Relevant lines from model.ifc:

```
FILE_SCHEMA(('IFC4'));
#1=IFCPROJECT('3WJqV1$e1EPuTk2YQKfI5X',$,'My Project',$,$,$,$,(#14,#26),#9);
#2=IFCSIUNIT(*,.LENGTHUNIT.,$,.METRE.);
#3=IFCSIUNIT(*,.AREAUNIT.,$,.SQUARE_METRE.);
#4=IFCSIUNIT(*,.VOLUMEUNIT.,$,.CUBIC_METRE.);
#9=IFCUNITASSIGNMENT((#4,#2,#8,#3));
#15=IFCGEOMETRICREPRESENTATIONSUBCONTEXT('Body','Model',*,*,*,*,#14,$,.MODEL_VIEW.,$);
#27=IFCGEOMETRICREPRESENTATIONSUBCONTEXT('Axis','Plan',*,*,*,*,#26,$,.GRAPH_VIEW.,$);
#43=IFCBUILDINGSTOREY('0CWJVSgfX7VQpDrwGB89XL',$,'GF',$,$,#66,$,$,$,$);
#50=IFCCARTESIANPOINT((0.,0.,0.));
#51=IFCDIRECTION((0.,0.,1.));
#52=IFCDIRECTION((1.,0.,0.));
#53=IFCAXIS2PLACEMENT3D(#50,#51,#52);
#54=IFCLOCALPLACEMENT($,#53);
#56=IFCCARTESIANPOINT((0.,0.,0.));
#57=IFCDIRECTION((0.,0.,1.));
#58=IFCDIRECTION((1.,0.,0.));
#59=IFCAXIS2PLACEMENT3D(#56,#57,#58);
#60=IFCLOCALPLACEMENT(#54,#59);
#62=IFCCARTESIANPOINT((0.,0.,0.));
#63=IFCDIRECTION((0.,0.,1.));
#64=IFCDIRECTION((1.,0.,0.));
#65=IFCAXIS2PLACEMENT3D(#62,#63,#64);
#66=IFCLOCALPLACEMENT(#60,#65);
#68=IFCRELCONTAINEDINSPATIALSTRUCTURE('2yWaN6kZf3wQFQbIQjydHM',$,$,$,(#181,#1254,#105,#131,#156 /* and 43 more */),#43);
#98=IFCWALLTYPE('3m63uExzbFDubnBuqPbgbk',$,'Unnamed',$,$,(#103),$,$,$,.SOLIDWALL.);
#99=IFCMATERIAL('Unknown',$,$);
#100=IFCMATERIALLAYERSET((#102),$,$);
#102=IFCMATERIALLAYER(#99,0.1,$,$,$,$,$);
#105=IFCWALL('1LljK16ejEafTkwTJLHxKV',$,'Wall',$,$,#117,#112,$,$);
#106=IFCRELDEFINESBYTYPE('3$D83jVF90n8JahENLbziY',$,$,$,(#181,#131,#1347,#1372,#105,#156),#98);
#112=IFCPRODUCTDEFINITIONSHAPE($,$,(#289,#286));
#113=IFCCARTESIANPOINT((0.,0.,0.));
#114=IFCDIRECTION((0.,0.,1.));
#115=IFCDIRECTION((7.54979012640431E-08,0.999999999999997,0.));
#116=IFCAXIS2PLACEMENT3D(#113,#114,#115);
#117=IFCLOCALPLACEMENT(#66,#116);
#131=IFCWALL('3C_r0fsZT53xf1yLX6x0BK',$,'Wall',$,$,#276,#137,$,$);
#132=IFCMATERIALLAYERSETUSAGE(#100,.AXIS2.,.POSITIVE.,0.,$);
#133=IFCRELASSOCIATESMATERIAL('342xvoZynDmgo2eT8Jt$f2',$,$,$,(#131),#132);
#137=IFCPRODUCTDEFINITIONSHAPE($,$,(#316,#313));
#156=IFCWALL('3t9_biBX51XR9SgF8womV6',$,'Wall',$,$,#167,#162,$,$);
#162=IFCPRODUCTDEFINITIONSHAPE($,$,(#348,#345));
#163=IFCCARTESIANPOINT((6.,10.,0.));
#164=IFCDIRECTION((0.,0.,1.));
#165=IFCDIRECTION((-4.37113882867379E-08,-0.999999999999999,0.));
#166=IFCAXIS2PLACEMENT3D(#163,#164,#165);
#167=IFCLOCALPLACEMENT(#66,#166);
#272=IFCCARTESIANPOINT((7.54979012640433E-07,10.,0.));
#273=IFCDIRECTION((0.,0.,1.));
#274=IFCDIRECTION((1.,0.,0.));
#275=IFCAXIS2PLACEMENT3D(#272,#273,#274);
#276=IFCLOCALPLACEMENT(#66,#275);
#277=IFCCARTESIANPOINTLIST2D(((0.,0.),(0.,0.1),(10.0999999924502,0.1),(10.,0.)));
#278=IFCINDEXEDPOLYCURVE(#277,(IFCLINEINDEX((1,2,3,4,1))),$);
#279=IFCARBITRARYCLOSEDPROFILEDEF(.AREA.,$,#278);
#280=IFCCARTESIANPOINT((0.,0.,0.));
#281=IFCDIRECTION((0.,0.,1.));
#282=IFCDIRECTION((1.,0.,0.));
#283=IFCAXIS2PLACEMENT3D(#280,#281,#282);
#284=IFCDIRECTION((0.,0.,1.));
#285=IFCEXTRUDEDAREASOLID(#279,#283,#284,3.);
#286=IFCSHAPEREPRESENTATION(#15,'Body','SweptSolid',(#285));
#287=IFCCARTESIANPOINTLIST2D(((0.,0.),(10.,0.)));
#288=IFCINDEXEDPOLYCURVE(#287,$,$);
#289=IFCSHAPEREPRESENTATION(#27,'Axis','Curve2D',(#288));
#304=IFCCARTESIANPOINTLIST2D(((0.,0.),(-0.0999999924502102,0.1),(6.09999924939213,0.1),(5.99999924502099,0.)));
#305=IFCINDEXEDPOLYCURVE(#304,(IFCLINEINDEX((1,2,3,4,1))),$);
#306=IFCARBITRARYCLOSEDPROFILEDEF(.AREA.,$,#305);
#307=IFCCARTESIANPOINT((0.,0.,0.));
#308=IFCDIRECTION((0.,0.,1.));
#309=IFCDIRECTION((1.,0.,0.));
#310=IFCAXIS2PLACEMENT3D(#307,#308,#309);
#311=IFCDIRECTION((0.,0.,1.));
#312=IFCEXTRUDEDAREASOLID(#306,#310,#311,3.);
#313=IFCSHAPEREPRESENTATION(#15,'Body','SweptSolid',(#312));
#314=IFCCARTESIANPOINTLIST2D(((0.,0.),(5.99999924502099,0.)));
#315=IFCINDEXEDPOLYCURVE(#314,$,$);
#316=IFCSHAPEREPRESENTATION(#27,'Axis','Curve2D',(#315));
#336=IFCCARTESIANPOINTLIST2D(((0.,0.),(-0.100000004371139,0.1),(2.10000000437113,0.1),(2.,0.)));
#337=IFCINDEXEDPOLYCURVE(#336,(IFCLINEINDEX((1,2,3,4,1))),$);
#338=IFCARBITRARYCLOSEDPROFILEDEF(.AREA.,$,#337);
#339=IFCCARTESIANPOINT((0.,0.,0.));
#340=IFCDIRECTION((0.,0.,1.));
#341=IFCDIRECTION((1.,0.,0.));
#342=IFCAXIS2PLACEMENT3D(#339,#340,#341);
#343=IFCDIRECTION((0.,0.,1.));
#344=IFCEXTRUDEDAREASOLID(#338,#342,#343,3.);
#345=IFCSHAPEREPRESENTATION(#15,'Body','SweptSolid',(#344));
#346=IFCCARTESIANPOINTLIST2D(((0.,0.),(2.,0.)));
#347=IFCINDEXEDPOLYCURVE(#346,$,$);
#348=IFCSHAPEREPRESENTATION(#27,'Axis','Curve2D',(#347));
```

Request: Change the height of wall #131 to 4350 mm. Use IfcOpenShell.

```python
import ifcopenshell
import ifcopenshell.geom
import ifcopenshell.util.representation
import ifcopenshell.util.shape

model = ifcopenshell.open("model.ifc")
settings = ifcopenshell.geom.settings()


def volume(element):
    """Net volume in cubic metres, openings subtracted."""
    shape = ifcopenshell.geom.create_shape(settings, element)
    return ifcopenshell.util.shape.get_volume(shape.geometry)


wall = model.by_id(131)
before = volume(wall)

body = ifcopenshell.util.representation.get_representation(wall, "Model", "Body")
solid = body.Items[0]
old_height = solid.Depth
solid.Depth = 4.35
after = volume(wall)

print(f"height {old_height:g} -> {solid.Depth:g}, volume {before:.3f} -> {after:.3f} m3")

model.write("model_rev.ifc")
```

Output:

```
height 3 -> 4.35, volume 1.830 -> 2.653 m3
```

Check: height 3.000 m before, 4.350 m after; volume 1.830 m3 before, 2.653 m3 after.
